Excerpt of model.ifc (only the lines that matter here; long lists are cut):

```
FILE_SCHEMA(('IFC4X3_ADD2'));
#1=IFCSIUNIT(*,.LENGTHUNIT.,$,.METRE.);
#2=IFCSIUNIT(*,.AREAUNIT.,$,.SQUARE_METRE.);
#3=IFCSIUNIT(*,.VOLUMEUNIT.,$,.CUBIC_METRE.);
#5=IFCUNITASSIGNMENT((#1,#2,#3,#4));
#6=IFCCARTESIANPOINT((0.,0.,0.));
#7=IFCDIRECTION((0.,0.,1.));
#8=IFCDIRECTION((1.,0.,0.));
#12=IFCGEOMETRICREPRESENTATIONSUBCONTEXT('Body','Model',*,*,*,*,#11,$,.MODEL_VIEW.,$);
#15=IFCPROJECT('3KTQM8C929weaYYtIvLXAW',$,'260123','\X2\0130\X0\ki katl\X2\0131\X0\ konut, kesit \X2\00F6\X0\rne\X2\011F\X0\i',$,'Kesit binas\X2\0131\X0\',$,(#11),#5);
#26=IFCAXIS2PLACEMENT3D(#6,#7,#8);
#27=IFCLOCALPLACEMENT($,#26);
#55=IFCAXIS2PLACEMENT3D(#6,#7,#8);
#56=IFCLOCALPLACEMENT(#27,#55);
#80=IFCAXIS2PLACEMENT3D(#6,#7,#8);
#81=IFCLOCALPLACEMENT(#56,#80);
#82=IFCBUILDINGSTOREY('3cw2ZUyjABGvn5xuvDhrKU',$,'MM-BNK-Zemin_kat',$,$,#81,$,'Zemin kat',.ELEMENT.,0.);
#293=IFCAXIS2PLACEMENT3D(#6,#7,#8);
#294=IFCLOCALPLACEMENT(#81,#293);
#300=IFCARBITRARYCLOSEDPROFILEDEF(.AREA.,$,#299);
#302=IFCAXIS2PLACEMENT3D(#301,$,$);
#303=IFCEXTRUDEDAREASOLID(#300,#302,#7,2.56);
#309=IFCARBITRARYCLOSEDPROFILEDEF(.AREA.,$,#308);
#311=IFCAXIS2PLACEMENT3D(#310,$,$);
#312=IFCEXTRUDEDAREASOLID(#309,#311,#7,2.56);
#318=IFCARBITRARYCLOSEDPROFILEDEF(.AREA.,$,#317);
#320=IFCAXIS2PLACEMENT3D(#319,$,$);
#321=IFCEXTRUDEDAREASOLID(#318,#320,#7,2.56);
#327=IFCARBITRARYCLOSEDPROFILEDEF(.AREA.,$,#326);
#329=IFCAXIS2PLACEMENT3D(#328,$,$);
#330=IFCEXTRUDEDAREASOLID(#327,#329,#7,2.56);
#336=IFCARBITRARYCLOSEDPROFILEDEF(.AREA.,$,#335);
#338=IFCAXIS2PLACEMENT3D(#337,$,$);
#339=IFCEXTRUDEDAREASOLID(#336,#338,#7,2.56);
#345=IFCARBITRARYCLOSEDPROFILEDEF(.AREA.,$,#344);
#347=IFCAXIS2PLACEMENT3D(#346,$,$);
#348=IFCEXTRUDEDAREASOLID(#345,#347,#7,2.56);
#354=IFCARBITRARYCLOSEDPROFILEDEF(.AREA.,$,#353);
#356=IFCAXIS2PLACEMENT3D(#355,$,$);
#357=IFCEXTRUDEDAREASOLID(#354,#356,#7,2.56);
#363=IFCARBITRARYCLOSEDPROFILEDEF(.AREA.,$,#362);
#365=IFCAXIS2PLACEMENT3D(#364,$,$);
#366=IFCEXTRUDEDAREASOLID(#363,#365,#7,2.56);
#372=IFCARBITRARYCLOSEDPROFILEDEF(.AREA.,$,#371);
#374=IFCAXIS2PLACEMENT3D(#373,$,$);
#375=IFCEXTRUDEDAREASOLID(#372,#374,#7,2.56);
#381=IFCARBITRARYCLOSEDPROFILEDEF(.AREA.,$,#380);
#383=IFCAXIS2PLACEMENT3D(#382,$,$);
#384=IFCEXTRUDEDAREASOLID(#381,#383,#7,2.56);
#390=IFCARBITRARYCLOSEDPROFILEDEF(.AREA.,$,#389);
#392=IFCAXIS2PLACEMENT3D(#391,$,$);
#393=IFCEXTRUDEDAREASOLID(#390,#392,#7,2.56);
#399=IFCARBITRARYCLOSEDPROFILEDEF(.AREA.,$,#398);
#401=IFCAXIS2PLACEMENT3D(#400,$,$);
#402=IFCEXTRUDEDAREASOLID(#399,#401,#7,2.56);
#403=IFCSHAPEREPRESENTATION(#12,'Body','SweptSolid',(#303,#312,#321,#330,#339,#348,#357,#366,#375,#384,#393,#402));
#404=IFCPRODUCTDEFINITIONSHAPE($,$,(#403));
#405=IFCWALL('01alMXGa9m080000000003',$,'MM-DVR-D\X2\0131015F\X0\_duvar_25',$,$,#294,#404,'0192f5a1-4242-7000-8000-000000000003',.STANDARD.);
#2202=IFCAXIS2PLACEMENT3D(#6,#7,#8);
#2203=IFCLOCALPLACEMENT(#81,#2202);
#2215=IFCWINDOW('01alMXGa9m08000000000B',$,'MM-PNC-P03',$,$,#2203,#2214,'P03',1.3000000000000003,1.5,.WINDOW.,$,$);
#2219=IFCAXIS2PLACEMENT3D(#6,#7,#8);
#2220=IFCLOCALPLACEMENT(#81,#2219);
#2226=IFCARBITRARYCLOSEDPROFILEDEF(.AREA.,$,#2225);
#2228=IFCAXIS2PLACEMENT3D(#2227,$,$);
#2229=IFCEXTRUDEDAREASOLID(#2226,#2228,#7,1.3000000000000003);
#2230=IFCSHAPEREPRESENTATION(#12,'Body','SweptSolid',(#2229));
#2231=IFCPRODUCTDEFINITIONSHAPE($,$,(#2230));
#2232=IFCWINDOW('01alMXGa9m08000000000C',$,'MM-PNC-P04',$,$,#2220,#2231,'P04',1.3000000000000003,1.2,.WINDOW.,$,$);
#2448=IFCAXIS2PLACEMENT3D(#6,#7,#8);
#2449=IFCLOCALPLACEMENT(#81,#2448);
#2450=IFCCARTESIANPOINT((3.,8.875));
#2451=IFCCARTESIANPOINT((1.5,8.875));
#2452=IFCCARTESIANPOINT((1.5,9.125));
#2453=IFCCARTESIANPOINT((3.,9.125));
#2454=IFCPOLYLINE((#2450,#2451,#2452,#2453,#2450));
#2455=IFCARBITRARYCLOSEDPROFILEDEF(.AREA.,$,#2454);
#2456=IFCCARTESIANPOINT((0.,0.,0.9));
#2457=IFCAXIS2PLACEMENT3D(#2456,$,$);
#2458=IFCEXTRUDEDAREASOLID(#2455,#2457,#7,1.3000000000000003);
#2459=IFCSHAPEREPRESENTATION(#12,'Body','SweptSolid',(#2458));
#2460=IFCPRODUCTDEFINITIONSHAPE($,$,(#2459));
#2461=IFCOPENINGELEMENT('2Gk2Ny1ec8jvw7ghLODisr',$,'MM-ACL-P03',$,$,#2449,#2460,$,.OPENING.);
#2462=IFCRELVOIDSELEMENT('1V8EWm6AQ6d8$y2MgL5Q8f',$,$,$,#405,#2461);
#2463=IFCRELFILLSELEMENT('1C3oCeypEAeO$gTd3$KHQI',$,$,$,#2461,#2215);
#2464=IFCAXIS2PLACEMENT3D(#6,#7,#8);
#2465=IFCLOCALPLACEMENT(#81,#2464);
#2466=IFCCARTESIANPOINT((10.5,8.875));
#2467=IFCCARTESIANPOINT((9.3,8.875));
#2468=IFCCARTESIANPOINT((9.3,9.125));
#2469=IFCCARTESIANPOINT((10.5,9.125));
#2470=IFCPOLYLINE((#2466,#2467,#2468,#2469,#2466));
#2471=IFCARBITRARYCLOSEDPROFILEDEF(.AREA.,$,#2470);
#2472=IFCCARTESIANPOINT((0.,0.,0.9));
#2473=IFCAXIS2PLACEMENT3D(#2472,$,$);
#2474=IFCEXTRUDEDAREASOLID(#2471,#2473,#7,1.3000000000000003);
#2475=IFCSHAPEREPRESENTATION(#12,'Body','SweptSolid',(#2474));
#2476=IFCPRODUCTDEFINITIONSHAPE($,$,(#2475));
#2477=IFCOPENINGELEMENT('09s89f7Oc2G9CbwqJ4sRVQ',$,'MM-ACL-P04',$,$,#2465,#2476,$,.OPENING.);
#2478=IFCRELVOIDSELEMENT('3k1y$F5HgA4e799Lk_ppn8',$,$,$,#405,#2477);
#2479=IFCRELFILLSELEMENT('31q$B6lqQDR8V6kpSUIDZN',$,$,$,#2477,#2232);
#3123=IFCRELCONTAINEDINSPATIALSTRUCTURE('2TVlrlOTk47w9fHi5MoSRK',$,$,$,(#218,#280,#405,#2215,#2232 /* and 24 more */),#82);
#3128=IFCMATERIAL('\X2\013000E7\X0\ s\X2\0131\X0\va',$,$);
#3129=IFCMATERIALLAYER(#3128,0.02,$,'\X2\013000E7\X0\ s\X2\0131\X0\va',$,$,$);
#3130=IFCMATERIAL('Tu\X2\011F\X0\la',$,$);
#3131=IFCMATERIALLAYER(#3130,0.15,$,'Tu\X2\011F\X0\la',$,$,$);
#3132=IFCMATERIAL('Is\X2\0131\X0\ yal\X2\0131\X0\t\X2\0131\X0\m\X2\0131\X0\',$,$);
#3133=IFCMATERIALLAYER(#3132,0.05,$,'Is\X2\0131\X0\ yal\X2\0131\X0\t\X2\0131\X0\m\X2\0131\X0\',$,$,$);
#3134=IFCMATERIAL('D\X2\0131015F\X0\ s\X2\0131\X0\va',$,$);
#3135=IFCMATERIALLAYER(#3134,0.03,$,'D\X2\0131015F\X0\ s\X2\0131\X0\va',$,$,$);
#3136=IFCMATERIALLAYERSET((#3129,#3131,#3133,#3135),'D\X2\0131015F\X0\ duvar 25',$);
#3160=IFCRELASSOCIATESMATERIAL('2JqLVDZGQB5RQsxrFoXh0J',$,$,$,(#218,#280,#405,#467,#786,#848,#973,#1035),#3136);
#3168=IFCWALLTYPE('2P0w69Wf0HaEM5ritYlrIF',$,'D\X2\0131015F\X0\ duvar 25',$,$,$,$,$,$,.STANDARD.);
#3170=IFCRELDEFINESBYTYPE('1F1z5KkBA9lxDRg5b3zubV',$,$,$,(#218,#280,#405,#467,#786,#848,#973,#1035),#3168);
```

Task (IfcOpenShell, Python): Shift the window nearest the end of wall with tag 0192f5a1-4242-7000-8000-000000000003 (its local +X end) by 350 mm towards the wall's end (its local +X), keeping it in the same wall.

```python
import ifcopenshell
import ifcopenshell.api.geometry
import ifcopenshell.util.placement
import ifcopenshell.util.unit

model = ifcopenshell.open("model.ifc")
unit_scale = ifcopenshell.util.unit.calculate_unit_scale(model)

window = model.by_id(2232)
opening = window.FillsVoids[0].RelatingOpeningElement
wall = opening.VoidsElements[0].RelatingBuildingElement

wall_matrix = ifcopenshell.util.placement.get_local_placement(wall.ObjectPlacement)
shift = wall_matrix[:3, 0] * 0.35 / unit_scale
before = ifcopenshell.util.placement.get_local_placement(window.ObjectPlacement)[:3, 3].copy()

# The window is not placed relative to its opening, so move both.
for product in (opening, window):
    matrix = ifcopenshell.util.placement.get_local_placement(product.ObjectPlacement)
    matrix[:3, 3] += shift
    ifcopenshell.api.geometry.edit_object_placement(model, product=product, matrix=matrix, is_si=False)

after = ifcopenshell.util.placement.get_local_placement(window.ObjectPlacement)[:3, 3]
print("window moved by", (after - before).round(3) + 0.0)

model.write("model_updated.ifc")
```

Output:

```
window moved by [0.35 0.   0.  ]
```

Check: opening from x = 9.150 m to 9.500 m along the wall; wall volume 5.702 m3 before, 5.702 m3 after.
